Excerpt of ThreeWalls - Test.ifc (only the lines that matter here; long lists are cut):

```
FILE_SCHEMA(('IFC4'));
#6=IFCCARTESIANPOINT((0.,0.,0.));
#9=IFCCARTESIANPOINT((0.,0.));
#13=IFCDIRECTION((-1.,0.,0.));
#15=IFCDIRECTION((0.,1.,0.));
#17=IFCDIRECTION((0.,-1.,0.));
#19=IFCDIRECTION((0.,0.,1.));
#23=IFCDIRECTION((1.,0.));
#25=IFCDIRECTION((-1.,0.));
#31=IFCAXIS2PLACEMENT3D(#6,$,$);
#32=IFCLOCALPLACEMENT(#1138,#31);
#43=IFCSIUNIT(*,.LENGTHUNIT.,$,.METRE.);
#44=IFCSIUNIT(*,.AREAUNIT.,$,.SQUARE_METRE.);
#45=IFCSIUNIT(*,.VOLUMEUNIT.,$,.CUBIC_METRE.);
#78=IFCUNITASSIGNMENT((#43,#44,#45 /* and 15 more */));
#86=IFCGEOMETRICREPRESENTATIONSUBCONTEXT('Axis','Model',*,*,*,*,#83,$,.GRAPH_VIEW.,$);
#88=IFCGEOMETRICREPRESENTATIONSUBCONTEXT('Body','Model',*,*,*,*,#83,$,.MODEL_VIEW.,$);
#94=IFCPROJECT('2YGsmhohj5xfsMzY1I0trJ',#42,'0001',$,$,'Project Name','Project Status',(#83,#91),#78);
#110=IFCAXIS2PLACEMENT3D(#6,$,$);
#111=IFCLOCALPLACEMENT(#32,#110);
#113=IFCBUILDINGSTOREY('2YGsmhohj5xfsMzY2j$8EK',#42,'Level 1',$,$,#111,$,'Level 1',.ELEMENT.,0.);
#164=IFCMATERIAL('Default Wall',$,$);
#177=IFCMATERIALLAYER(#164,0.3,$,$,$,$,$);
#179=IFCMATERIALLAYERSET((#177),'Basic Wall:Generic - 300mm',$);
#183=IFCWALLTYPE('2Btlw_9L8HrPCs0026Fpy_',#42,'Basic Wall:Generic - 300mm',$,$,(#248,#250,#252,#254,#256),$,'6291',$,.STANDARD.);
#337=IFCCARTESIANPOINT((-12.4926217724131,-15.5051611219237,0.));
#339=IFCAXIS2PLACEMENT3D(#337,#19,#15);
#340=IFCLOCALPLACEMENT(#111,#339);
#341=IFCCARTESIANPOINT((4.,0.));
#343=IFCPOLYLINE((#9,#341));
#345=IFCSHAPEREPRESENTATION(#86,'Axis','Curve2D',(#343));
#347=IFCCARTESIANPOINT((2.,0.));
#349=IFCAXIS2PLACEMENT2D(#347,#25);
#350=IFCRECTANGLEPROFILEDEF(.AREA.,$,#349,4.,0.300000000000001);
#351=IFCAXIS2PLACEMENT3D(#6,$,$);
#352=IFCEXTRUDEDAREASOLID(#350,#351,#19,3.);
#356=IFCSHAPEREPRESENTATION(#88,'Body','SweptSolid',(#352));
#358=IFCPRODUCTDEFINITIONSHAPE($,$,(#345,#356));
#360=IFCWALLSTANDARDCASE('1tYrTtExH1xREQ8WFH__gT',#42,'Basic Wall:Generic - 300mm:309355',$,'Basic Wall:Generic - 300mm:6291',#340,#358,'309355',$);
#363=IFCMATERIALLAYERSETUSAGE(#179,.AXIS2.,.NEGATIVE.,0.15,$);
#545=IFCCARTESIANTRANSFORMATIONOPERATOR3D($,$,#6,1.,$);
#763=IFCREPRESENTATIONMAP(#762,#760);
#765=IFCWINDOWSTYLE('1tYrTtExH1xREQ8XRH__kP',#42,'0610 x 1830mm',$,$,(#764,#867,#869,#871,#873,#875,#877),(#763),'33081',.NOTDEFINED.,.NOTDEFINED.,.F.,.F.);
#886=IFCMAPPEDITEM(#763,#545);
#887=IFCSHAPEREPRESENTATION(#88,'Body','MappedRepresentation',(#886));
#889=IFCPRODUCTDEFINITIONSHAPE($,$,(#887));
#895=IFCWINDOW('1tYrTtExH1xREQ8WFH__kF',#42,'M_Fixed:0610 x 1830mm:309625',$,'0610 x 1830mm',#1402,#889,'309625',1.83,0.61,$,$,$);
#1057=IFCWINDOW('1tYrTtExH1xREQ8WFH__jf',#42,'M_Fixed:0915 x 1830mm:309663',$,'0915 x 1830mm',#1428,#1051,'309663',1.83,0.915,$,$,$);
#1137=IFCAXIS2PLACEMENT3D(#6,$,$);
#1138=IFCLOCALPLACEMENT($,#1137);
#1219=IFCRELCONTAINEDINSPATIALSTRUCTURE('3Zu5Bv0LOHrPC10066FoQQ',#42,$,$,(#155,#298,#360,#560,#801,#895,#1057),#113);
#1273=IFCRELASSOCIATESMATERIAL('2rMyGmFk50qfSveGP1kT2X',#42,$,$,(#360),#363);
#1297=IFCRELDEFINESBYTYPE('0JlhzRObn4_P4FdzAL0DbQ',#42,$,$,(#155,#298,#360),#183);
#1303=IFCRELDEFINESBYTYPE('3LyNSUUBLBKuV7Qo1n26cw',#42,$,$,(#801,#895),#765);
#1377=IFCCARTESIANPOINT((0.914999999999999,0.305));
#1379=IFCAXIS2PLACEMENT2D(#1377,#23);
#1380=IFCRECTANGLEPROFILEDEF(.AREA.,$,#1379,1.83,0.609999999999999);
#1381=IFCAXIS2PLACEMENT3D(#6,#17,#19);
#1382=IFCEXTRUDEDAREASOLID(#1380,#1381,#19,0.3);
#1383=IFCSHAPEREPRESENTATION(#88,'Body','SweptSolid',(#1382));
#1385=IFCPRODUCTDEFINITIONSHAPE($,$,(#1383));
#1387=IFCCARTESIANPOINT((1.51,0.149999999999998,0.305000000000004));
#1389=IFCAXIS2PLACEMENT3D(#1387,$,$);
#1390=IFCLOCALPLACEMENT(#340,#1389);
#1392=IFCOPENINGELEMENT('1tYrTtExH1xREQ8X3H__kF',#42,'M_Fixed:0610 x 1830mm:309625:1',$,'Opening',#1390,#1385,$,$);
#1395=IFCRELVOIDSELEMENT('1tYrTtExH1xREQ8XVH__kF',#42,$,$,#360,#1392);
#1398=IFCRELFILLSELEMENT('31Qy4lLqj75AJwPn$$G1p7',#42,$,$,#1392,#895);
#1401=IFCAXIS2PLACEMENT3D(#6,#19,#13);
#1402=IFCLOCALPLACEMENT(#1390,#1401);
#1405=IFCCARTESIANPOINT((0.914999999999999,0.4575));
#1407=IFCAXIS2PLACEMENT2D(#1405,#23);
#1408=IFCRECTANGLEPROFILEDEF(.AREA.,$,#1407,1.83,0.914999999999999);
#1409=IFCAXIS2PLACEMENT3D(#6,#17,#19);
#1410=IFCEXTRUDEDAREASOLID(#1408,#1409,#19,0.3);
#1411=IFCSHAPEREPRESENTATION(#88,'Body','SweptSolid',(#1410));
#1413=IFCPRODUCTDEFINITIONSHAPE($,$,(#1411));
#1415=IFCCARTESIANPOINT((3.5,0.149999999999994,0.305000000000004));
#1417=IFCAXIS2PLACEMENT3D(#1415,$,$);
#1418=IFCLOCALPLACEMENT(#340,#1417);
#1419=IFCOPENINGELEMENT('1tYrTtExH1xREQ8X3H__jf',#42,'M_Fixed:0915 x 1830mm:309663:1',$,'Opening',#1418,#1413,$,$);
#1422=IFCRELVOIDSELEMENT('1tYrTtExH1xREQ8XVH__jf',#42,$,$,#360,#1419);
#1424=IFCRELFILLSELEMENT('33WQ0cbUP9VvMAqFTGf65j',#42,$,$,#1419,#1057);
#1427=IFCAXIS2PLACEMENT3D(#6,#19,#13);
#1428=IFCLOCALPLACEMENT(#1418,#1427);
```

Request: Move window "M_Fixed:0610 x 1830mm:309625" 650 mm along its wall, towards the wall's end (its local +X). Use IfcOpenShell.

```python
import ifcopenshell
import ifcopenshell.api.geometry
import ifcopenshell.util.placement

model = ifcopenshell.open("ThreeWalls - Test.ifc")

window = model.by_guid("1tYrTtExH1xREQ8WFH__kF")
opening = window.FillsVoids[0].RelatingOpeningElement
wall = opening.VoidsElements[0].RelatingBuildingElement

wall_matrix = ifcopenshell.util.placement.get_local_placement(wall.ObjectPlacement)
shift = wall_matrix[:3, 0] * 0.65
before = ifcopenshell.util.placement.get_local_placement(window.ObjectPlacement)[:3, 3].copy()

# The window is placed relative to its opening, so it follows when the opening moves.
matrix = ifcopenshell.util.placement.get_local_placement(opening.ObjectPlacement)
matrix[:3, 3] += shift
ifcopenshell.api.geometry.edit_object_placement(
    model, product=opening, matrix=matrix, is_si=False, should_transform_children=True
)

after = ifcopenshell.util.placement.get_local_placement(window.ObjectPlacement)[:3, 3]
print("window moved by", (after - before).round(3) + 0.0)

model.write("ThreeWalls - Test_updated.ifc")
```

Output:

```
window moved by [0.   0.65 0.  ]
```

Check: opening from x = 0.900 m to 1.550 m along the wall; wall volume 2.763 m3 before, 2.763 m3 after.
